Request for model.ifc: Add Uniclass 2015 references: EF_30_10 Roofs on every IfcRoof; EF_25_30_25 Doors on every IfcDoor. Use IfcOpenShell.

First a look at what the model holds.

```python
import ifcopenshell

model = ifcopenshell.open("model.ifc")
print(model.schema)
print("classifications:", [c.Name for c in model.by_type("IfcClassification")])
for ifc_class in ("IfcDoor", "IfcRoof", "IfcStair", "IfcWall", "IfcWindow"):
    print(ifc_class, len(model.by_type(ifc_class)))
```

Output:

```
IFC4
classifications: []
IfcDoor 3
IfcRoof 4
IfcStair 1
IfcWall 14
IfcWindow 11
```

```python
import ifcopenshell
import ifcopenshell.api.classification

model = ifcopenshell.open("model.ifc")

system = ifcopenshell.api.classification.add_classification(model, classification="Uniclass 2015")

codes = {
    "IfcRoof": ("EF_30_10", "Roofs"),
    "IfcDoor": ("EF_25_30_25", "Doors"),
}
for ifc_class, (code, name) in codes.items():
    products = model.by_type(ifc_class)
    ifcopenshell.api.classification.add_reference(
        model, products=products, classification=system, identification=code, name=name
    )
    print(code, len(products))

model.write("model_updated.ifc")
```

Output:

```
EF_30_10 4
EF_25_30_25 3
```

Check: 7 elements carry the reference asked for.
